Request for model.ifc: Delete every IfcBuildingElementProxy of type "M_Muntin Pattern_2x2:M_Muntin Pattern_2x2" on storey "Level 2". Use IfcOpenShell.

First a look at what the model holds.

```python
import ifcopenshell
import ifcopenshell.util.element

model = ifcopenshell.open("model.ifc")
print(model.schema)
storey = next(s for s in model.by_type("IfcBuildingStorey") if s.Name == "Level 2")
proxies = [e for e in ifcopenshell.util.element.get_decomposition(storey) if e.is_a("IfcBuildingElementProxy")]
seen = {}
for e in proxies:
    element_type = ifcopenshell.util.element.get_type(e)
    name = element_type.Name if element_type not in (None, e) else None
    seen[name] = seen.get(name, 0) + 1
for name, count in sorted(seen.items(), key=str):
    print(count, "x", name)
```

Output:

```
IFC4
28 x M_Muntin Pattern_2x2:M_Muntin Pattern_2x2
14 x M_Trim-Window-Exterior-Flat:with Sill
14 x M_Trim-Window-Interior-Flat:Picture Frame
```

```python
import ifcopenshell
import ifcopenshell.api.root
import ifcopenshell.util.element

model = ifcopenshell.open("model.ifc")

storey = next(s for s in model.by_type("IfcBuildingStorey") if s.Name == "Level 2")
proxies = [e for e in ifcopenshell.util.element.get_decomposition(storey) if e.is_a("IfcBuildingElementProxy")]
targets = [e for e in proxies if (t := ifcopenshell.util.element.get_type(e)) not in (None, e) and t.Name == "M_Muntin Pattern_2x2:M_Muntin Pattern_2x2"]

for e in targets:
    ifcopenshell.api.root.remove_product(model, product=e)
print(len(targets), "removed")

model.write("model_updated.ifc")
```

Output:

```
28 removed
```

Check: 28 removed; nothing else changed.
